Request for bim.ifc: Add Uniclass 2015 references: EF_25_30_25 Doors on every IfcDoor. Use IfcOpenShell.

First a look at what the model holds.

```python
import ifcopenshell

model = ifcopenshell.open("bim.ifc")
print(model.schema)
print("classifications:", [c.Name for c in model.by_type("IfcClassification")])
for ifc_class in ("IfcDoor", "IfcRoof", "IfcStair", "IfcWall", "IfcWindow"):
    print(ifc_class, len(model.by_type(ifc_class)))
```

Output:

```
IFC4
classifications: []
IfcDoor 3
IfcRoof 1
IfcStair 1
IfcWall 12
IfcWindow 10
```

```python
import ifcopenshell
import ifcopenshell.api.classification

model = ifcopenshell.open("bim.ifc")

system = ifcopenshell.api.classification.add_classification(model, classification="Uniclass 2015")

codes = {
    "IfcDoor": ("EF_25_30_25", "Doors"),
}
for ifc_class, (code, name) in codes.items():
    products = model.by_type(ifc_class)
    ifcopenshell.api.classification.add_reference(
        model, products=products, classification=system, identification=code, name=name
    )
    print(code, len(products))

model.write("bim_v2.ifc")
```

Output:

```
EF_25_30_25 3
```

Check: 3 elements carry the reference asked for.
